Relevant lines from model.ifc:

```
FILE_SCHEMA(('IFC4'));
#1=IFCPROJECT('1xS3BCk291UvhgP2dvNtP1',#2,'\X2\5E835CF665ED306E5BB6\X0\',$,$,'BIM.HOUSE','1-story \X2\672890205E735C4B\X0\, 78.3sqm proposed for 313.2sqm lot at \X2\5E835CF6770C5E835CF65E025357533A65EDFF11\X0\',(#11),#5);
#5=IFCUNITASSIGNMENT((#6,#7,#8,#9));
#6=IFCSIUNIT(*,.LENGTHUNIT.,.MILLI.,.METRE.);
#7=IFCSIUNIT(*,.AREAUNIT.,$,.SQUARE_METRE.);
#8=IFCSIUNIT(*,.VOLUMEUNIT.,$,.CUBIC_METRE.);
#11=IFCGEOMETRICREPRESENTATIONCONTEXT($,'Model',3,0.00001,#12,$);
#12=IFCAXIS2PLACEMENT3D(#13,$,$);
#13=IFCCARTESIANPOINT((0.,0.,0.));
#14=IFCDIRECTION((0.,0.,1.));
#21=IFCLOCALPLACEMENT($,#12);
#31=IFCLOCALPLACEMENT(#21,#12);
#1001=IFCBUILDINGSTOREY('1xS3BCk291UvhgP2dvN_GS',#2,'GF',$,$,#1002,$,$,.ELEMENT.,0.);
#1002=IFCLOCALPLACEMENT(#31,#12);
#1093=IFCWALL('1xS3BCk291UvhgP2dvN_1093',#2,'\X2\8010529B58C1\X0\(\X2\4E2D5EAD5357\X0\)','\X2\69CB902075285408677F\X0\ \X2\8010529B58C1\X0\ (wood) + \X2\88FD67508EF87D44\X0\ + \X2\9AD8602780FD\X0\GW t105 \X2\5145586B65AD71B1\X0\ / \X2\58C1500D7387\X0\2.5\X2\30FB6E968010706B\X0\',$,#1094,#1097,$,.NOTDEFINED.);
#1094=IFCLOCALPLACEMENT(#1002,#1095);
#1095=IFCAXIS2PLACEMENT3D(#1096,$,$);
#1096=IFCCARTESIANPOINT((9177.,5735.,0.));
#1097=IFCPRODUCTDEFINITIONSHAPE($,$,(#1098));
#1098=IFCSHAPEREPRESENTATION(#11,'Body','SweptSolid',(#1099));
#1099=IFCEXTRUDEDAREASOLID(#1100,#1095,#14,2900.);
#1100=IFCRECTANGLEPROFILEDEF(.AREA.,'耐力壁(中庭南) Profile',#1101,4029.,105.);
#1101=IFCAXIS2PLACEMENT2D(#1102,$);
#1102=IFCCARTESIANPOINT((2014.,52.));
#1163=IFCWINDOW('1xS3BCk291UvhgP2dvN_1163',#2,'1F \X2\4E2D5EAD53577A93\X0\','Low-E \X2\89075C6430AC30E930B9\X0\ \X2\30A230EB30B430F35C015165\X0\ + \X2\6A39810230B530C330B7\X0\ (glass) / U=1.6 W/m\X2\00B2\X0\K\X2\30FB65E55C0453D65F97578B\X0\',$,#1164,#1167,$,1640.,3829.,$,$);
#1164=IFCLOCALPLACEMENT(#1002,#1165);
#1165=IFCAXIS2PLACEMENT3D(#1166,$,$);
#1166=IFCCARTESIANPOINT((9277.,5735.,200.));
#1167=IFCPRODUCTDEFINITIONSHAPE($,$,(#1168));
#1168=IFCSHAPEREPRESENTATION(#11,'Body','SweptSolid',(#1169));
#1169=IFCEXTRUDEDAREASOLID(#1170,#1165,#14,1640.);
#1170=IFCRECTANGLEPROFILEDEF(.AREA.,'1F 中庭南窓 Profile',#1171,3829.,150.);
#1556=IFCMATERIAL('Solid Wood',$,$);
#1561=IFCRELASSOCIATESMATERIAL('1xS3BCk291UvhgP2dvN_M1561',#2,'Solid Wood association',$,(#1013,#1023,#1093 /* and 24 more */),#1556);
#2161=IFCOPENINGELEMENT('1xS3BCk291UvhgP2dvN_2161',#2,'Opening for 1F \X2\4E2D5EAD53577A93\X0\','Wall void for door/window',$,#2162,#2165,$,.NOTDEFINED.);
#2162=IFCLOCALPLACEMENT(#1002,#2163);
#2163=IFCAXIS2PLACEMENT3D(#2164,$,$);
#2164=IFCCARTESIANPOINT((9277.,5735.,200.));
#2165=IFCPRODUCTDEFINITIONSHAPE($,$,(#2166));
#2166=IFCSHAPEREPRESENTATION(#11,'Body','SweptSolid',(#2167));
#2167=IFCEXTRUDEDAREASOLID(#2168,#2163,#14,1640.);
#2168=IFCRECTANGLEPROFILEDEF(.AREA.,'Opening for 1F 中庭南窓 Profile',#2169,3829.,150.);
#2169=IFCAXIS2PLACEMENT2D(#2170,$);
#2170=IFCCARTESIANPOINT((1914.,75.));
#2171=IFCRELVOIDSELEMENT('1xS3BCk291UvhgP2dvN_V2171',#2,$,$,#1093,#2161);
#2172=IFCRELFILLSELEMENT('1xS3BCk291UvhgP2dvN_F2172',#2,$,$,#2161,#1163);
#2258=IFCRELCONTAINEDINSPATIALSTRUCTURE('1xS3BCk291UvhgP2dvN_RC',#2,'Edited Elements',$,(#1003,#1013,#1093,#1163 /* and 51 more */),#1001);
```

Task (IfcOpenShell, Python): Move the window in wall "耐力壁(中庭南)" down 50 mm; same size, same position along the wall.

```python
import numpy as np
import ifcopenshell
import ifcopenshell.api.geometry
import ifcopenshell.util.placement
import ifcopenshell.util.unit

model = ifcopenshell.open("model.ifc")
unit_scale = ifcopenshell.util.unit.calculate_unit_scale(model)

window = model.by_guid("1xS3BCk291UvhgP2dvN_1163")
opening = window.FillsVoids[0].RelatingOpeningElement
dz = -0.05 / unit_scale

shift = np.array([0.0, 0.0, dz])
# The window is not placed relative to its opening, so move both.
for product in (opening, window):
    matrix = ifcopenshell.util.placement.get_local_placement(product.ObjectPlacement)
    matrix[:3, 3] += shift
    ifcopenshell.api.geometry.edit_object_placement(model, product=product, matrix=matrix, is_si=False)

print(f"moved by {dz * unit_scale:+.3f} m")

model.write("model_edited.ifc")
```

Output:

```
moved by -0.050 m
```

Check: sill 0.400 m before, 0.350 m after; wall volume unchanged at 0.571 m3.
